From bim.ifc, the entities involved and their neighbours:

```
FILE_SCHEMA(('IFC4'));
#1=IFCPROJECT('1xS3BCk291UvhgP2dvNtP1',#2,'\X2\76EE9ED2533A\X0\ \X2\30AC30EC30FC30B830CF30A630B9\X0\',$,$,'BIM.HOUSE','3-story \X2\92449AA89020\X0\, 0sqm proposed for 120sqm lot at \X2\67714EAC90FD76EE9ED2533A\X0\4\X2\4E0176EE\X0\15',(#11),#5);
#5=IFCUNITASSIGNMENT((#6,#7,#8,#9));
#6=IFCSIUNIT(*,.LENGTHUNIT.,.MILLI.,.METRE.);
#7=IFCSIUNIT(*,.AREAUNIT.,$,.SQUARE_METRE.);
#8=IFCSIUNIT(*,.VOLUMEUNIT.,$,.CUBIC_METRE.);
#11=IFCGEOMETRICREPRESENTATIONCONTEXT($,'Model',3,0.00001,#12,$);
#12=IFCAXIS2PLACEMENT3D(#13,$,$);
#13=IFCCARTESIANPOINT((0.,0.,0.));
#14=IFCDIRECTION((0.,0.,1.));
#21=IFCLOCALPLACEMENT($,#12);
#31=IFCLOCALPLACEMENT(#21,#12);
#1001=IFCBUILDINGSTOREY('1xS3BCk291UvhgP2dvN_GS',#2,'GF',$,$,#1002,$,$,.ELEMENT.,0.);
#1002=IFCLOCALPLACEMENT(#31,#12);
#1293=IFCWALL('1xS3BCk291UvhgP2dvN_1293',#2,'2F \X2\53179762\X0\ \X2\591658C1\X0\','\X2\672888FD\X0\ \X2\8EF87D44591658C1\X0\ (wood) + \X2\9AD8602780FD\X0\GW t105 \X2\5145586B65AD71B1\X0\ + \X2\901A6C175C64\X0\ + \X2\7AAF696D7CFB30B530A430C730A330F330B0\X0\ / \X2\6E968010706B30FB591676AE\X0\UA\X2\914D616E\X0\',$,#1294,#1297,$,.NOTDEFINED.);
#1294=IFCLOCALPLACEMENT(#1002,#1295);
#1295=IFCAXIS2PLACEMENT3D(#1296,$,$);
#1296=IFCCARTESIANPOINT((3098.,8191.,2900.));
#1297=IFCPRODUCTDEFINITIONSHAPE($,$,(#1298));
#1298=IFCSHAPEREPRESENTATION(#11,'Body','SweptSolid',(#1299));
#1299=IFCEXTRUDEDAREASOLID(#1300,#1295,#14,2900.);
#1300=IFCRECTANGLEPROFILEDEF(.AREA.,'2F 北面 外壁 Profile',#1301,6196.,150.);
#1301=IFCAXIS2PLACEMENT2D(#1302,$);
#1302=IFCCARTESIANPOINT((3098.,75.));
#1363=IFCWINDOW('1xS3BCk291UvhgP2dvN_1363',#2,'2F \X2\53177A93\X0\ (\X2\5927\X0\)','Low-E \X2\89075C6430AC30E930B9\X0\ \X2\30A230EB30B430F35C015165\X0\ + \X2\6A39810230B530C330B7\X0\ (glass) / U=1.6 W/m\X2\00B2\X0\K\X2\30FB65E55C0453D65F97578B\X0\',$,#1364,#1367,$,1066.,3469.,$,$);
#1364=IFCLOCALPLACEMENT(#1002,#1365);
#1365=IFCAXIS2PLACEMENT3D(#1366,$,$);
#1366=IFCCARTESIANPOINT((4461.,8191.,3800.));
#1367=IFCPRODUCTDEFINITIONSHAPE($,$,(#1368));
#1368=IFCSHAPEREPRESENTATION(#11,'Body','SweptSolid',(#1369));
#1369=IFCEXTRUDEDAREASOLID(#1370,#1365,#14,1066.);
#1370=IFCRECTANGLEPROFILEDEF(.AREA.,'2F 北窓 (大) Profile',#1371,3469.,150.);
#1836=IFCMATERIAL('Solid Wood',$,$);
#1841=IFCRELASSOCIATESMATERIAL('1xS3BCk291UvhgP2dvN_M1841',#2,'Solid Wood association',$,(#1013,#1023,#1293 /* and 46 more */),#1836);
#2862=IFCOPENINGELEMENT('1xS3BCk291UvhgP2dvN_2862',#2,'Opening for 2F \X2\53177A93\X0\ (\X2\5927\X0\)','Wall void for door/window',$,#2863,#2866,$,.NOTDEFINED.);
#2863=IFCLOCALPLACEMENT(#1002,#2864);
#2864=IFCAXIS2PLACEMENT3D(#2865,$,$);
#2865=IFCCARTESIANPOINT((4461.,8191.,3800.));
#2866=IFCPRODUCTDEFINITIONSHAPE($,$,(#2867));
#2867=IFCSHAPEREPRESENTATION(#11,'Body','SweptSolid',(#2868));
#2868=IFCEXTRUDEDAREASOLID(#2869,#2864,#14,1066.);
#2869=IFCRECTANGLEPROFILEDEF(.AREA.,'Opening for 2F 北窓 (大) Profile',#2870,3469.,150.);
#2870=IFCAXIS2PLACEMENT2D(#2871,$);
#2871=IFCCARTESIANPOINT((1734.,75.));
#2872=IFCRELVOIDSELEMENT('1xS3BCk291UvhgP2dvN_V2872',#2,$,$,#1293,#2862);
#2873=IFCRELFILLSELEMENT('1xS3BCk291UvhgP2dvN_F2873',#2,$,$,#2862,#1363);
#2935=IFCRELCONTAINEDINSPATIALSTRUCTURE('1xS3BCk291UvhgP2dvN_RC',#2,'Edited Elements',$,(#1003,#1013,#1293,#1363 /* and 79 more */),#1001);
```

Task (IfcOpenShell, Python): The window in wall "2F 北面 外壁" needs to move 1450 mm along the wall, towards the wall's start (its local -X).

```python
import ifcopenshell
import ifcopenshell.api.geometry
import ifcopenshell.util.placement

model = ifcopenshell.open("bim.ifc")

window = model.by_guid("1xS3BCk291UvhgP2dvN_1363")
opening = window.FillsVoids[0].RelatingOpeningElement
wall = opening.VoidsElements[0].RelatingBuildingElement

wall_matrix = ifcopenshell.util.placement.get_local_placement(wall.ObjectPlacement)
shift = wall_matrix[:3, 0] * -1450.0
before = ifcopenshell.util.placement.get_local_placement(window.ObjectPlacement)[:3, 3].copy()

# The window is not placed relative to its opening, so move both.
for product in (opening, window):
    matrix = ifcopenshell.util.placement.get_local_placement(product.ObjectPlacement)
    matrix[:3, 3] += shift
    ifcopenshell.api.geometry.edit_object_placement(model, product=product, matrix=matrix, is_si=False)

after = ifcopenshell.util.placement.get_local_placement(window.ObjectPlacement)[:3, 3]
print("window moved by", (after - before).round(3) + 0.0)

model.write("bim_v2.ifc")
```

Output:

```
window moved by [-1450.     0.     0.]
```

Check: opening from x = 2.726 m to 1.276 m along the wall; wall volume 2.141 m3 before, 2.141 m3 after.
